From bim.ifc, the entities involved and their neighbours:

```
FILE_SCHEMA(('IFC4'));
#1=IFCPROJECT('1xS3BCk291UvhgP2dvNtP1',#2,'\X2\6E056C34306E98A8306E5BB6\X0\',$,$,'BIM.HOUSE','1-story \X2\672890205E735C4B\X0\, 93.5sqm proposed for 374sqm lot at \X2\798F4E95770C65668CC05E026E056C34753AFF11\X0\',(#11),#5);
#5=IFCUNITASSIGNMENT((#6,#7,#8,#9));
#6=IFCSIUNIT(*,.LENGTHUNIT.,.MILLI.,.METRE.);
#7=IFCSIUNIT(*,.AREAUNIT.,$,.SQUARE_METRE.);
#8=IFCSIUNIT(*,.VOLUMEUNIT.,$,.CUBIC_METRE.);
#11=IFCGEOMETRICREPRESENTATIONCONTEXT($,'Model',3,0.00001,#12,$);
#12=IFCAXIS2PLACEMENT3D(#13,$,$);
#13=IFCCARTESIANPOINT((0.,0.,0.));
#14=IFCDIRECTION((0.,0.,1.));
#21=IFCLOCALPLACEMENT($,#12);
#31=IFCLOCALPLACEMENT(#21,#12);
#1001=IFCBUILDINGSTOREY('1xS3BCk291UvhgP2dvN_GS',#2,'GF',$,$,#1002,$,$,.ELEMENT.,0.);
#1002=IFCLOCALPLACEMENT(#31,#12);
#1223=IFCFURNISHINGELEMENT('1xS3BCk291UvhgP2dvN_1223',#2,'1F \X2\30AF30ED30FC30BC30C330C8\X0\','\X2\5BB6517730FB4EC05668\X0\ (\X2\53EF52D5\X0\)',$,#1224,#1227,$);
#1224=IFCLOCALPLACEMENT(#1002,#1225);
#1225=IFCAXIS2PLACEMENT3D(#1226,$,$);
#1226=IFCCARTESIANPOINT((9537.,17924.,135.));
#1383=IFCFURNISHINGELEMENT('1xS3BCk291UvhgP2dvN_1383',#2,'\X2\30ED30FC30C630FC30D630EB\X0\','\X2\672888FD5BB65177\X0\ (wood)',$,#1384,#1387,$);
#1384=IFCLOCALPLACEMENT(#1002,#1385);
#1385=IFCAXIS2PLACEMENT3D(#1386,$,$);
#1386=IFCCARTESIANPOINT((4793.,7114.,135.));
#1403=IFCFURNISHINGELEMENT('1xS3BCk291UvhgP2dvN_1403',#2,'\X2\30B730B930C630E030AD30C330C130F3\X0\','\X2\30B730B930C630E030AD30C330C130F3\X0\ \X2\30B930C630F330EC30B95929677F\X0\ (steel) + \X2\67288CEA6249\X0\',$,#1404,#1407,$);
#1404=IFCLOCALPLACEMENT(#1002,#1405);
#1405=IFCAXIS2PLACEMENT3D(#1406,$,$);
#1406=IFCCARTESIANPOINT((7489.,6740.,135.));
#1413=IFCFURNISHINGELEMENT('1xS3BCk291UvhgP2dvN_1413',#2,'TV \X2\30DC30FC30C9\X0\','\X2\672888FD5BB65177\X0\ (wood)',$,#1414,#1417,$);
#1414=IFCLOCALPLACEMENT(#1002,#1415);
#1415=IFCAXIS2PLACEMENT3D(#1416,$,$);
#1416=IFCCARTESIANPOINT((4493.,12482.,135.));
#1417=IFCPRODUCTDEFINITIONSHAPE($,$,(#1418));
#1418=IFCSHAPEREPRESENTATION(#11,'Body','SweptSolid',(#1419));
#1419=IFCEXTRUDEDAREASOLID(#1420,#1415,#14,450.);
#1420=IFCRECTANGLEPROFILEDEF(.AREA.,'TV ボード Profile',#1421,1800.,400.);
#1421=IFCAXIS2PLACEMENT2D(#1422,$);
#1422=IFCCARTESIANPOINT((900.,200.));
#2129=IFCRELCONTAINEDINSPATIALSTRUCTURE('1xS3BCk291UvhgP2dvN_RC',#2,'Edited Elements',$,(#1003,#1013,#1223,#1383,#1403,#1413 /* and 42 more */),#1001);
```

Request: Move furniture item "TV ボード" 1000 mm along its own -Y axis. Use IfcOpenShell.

```python
import ifcopenshell
import ifcopenshell.api.geometry
import ifcopenshell.util.placement

model = ifcopenshell.open("bim.ifc")

item = model.by_id(1413)
matrix = ifcopenshell.util.placement.get_local_placement(item.ObjectPlacement)
matrix[:3, 3] -= matrix[:3, 1] * 1000.0
ifcopenshell.api.geometry.edit_object_placement(model, product=item, matrix=matrix, is_si=False)

print(ifcopenshell.util.placement.get_local_placement(item.ObjectPlacement).round(3) + 0.0)

model.write("bim_rev.ifc")
```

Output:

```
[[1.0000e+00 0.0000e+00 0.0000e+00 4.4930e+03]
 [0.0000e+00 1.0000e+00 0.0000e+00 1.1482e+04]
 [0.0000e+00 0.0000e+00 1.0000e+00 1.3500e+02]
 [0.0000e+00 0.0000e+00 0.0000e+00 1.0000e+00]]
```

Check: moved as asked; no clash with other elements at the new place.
